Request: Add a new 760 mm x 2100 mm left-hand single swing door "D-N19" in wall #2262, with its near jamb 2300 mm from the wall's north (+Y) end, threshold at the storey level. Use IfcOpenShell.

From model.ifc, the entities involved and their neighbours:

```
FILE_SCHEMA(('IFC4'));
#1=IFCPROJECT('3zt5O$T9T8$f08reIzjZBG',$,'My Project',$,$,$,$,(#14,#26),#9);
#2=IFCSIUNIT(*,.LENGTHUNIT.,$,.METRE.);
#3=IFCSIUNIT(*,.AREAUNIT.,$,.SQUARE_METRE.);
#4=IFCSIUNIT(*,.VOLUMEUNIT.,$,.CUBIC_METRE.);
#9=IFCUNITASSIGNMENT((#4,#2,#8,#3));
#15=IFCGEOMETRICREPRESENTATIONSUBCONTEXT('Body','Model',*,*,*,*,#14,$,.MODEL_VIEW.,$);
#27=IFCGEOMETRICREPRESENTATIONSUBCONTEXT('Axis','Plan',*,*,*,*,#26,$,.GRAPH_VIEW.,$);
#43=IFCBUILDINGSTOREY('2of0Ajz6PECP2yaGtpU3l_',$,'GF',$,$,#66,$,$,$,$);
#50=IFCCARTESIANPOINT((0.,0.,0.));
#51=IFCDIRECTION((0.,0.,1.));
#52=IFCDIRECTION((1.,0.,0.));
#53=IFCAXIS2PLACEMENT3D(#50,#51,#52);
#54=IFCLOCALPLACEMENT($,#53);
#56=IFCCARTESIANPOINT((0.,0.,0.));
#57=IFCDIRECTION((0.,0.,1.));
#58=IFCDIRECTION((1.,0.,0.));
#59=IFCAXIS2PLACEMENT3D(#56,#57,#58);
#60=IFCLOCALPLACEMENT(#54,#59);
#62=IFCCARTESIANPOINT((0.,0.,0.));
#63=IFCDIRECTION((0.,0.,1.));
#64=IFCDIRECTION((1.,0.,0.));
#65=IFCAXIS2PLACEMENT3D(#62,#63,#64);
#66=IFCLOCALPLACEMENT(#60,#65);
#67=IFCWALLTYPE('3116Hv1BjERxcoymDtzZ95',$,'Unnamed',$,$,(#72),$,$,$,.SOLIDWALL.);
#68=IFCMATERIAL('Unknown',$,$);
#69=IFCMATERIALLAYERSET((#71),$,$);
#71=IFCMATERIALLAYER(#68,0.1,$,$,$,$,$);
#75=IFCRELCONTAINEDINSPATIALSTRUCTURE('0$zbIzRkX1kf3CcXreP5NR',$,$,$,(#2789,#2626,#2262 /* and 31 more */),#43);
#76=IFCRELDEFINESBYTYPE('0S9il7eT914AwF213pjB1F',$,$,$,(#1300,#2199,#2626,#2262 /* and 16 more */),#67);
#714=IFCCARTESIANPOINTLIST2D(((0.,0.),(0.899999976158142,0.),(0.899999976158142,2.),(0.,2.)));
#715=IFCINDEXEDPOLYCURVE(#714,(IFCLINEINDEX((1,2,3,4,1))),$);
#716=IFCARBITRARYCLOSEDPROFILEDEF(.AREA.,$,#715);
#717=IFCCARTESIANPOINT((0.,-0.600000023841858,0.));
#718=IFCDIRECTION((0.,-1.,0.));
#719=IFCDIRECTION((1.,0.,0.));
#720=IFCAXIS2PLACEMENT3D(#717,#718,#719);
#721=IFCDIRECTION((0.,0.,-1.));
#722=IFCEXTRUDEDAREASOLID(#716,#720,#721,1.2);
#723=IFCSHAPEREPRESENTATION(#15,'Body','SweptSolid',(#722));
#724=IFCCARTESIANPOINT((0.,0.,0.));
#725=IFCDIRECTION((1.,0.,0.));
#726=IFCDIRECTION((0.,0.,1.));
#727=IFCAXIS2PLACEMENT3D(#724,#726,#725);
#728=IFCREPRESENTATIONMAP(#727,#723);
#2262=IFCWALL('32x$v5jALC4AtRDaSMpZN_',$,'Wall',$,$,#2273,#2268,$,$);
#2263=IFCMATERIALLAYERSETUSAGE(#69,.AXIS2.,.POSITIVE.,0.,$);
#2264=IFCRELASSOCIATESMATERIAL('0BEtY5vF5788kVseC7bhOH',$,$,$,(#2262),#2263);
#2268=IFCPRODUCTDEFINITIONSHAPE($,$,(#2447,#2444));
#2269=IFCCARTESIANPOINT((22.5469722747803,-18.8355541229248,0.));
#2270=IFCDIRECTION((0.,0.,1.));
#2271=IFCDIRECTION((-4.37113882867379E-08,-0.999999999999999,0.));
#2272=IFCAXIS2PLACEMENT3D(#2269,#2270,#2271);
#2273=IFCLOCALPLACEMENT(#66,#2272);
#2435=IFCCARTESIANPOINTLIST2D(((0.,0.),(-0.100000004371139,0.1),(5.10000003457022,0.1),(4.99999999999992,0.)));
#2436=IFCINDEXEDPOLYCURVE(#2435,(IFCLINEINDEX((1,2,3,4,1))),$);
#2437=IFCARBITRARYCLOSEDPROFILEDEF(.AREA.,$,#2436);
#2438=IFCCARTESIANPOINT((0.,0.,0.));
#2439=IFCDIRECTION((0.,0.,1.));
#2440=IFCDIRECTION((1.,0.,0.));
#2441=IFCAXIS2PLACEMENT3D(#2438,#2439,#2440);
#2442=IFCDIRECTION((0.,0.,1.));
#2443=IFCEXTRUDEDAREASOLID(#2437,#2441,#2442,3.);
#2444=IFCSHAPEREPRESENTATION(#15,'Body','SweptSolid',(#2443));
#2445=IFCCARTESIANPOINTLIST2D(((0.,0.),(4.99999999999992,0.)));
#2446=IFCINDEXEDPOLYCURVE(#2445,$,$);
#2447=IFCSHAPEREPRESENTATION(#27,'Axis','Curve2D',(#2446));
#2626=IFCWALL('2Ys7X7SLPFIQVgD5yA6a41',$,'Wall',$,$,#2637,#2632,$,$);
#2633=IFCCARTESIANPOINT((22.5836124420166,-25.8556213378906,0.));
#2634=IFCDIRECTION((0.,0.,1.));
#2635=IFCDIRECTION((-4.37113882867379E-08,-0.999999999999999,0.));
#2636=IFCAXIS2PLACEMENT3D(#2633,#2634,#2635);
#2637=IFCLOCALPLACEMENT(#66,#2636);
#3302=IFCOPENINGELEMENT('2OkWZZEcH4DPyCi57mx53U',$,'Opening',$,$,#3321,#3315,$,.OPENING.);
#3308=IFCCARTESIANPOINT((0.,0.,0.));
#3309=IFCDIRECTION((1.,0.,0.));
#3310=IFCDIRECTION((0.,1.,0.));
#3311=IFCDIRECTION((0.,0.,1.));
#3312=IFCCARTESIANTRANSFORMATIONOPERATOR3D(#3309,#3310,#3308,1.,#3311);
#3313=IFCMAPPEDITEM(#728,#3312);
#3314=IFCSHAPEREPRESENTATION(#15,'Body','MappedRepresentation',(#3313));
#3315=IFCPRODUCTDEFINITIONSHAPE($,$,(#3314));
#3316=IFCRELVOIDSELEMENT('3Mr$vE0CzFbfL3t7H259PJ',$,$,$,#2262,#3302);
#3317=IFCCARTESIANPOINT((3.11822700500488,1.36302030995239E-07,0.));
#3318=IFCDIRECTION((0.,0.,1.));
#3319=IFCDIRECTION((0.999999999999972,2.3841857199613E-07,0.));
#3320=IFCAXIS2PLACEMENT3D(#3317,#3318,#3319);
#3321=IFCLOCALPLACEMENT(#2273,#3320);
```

```python
import numpy as np
import ifcopenshell
import ifcopenshell.api.feature
import ifcopenshell.api.geometry
import ifcopenshell.api.root
import ifcopenshell.api.spatial
import ifcopenshell.geom
import ifcopenshell.util.element
import ifcopenshell.util.placement
import ifcopenshell.util.representation
import ifcopenshell.util.shape
import ifcopenshell.util.unit

model = ifcopenshell.open("model.ifc")
unit_scale = ifcopenshell.util.unit.calculate_unit_scale(model)
settings = ifcopenshell.geom.settings()


def volume(element):
    """Net volume in cubic metres, openings subtracted."""
    shape = ifcopenshell.geom.create_shape(settings, element)
    return ifcopenshell.util.shape.get_volume(shape.geometry)


wall = model.by_guid("32x$v5jALC4AtRDaSMpZN_")
storey = ifcopenshell.util.element.get_container(wall, ifc_class="IfcBuildingStorey")
context = ifcopenshell.util.representation.get_context(model, "Model", "Body", "MODEL_VIEW")
before = volume(wall)

width, height, from_end, sill = 0.76, 2.1, 2.3, 0.0  # metres

# The wall runs along its own X axis, and the end named is its -X end.
wall_shape = ifcopenshell.geom.create_shape(settings, wall)
x, y, z = ifcopenshell.util.shape.get_vertices(wall_shape.geometry).T
start = x.min() + from_end
face, thickness = float(y.min()), float(y.max() - y.min())
wall_matrix = ifcopenshell.util.placement.get_local_placement(wall.ObjectPlacement)
level = ifcopenshell.util.placement.get_local_placement(storey.ObjectPlacement)[2, 3]


def in_wall(x, y):
    """Placement at x, y metres in the wall's axes, at sill height."""
    matrix = wall_matrix.copy()
    matrix[:, 3] = wall_matrix @ np.array([x / unit_scale, y / unit_scale, 0.0, 1.0])
    matrix[2, 3] = level + sill / unit_scale
    return matrix


# Opening: a box that overshoots both wall faces by 50 mm.
opening = ifcopenshell.api.root.create_entity(model, ifc_class="IfcOpeningElement", predefined_type="OPENING")
box = ifcopenshell.api.geometry.add_wall_representation(
    model, context=context, length=width, height=height, thickness=thickness + 0.1
)
ifcopenshell.api.geometry.assign_representation(model, product=opening, representation=box)
ifcopenshell.api.geometry.edit_object_placement(model, product=opening, matrix=in_wall(start, face - 0.05), is_si=False)
ifcopenshell.api.feature.add_feature(model, feature=opening, element=wall)

door = ifcopenshell.api.root.create_entity(model, ifc_class="IfcDoor", name="D-N19", predefined_type="DOOR")
door.OverallWidth, door.OverallHeight = width / unit_scale, height / unit_scale
door.OperationType = "SINGLE_SWING_LEFT"
body = ifcopenshell.api.geometry.add_door_representation(
    model,
    context=context,
    overall_width=door.OverallWidth,
    overall_height=door.OverallHeight,
    operation_type="SINGLE_SWING_LEFT",
    lining_properties={"LiningDepth": thickness / unit_scale, "ThresholdDepth": thickness / unit_scale},
)
ifcopenshell.api.geometry.assign_representation(model, product=door, representation=body)
ifcopenshell.api.spatial.assign_container(model, products=[door], relating_structure=storey)
ifcopenshell.api.feature.add_filling(model, opening=opening, element=door)

# The lining spans the wall, so the door starts at the wall face.
ifcopenshell.api.geometry.edit_object_placement(model, product=door, matrix=in_wall(start, face), is_si=False)

after = volume(wall)

print(f"wall volume {before:.3f} -> {after:.3f} m3")

model.write("model_updated.ifc")
```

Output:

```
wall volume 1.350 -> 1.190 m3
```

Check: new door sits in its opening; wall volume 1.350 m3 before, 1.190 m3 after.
